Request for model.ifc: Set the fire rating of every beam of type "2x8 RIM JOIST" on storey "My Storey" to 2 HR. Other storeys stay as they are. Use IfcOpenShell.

First a look at what the model holds.

```python
import ifcopenshell
import ifcopenshell.util.element

model = ifcopenshell.open("model.ifc")
print(model.schema)
storey = next(s for s in model.by_type("IfcBuildingStorey") if s.Name == "My Storey")
beams = [e for e in ifcopenshell.util.element.get_decomposition(storey) if e.is_a("IfcBeam")]
seen = {}
for e in beams:
    element_type = ifcopenshell.util.element.get_type(e)
    key = (element_type.Name if element_type != e and element_type else None, ifcopenshell.util.element.get_pset(e, "Pset_BeamCommon", "FireRating"))
    seen[key] = seen.get(key, 0) + 1
for (name, value), count in sorted(seen.items(), key=str):
    print(count, "x", name, "|", value)
```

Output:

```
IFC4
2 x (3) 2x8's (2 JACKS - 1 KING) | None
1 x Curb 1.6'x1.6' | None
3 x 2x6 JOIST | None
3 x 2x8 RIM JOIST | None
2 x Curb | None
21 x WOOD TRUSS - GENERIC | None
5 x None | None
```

```python
import ifcopenshell
import ifcopenshell.api.pset
import ifcopenshell.util.element

model = ifcopenshell.open("model.ifc")

storey = next(s for s in model.by_type("IfcBuildingStorey") if s.Name == "My Storey")
beams = [e for e in ifcopenshell.util.element.get_decomposition(storey) if e.is_a("IfcBeam")]

count = 0
for e in beams:
    element_type = ifcopenshell.util.element.get_type(e)
    if element_type in (None, e) or element_type.Name != "2x8 RIM JOIST":
        continue
    # add_pset returns the element's existing set when there is one.
    pset = ifcopenshell.api.pset.add_pset(model, product=e, name="Pset_BeamCommon")
    ifcopenshell.api.pset.edit_pset(model, pset=pset, properties={"FireRating": "2 HR"})
    count += 1

print(count, "beams updated")

model.write("model_v2.ifc")
```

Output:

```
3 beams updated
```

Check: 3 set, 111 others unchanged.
